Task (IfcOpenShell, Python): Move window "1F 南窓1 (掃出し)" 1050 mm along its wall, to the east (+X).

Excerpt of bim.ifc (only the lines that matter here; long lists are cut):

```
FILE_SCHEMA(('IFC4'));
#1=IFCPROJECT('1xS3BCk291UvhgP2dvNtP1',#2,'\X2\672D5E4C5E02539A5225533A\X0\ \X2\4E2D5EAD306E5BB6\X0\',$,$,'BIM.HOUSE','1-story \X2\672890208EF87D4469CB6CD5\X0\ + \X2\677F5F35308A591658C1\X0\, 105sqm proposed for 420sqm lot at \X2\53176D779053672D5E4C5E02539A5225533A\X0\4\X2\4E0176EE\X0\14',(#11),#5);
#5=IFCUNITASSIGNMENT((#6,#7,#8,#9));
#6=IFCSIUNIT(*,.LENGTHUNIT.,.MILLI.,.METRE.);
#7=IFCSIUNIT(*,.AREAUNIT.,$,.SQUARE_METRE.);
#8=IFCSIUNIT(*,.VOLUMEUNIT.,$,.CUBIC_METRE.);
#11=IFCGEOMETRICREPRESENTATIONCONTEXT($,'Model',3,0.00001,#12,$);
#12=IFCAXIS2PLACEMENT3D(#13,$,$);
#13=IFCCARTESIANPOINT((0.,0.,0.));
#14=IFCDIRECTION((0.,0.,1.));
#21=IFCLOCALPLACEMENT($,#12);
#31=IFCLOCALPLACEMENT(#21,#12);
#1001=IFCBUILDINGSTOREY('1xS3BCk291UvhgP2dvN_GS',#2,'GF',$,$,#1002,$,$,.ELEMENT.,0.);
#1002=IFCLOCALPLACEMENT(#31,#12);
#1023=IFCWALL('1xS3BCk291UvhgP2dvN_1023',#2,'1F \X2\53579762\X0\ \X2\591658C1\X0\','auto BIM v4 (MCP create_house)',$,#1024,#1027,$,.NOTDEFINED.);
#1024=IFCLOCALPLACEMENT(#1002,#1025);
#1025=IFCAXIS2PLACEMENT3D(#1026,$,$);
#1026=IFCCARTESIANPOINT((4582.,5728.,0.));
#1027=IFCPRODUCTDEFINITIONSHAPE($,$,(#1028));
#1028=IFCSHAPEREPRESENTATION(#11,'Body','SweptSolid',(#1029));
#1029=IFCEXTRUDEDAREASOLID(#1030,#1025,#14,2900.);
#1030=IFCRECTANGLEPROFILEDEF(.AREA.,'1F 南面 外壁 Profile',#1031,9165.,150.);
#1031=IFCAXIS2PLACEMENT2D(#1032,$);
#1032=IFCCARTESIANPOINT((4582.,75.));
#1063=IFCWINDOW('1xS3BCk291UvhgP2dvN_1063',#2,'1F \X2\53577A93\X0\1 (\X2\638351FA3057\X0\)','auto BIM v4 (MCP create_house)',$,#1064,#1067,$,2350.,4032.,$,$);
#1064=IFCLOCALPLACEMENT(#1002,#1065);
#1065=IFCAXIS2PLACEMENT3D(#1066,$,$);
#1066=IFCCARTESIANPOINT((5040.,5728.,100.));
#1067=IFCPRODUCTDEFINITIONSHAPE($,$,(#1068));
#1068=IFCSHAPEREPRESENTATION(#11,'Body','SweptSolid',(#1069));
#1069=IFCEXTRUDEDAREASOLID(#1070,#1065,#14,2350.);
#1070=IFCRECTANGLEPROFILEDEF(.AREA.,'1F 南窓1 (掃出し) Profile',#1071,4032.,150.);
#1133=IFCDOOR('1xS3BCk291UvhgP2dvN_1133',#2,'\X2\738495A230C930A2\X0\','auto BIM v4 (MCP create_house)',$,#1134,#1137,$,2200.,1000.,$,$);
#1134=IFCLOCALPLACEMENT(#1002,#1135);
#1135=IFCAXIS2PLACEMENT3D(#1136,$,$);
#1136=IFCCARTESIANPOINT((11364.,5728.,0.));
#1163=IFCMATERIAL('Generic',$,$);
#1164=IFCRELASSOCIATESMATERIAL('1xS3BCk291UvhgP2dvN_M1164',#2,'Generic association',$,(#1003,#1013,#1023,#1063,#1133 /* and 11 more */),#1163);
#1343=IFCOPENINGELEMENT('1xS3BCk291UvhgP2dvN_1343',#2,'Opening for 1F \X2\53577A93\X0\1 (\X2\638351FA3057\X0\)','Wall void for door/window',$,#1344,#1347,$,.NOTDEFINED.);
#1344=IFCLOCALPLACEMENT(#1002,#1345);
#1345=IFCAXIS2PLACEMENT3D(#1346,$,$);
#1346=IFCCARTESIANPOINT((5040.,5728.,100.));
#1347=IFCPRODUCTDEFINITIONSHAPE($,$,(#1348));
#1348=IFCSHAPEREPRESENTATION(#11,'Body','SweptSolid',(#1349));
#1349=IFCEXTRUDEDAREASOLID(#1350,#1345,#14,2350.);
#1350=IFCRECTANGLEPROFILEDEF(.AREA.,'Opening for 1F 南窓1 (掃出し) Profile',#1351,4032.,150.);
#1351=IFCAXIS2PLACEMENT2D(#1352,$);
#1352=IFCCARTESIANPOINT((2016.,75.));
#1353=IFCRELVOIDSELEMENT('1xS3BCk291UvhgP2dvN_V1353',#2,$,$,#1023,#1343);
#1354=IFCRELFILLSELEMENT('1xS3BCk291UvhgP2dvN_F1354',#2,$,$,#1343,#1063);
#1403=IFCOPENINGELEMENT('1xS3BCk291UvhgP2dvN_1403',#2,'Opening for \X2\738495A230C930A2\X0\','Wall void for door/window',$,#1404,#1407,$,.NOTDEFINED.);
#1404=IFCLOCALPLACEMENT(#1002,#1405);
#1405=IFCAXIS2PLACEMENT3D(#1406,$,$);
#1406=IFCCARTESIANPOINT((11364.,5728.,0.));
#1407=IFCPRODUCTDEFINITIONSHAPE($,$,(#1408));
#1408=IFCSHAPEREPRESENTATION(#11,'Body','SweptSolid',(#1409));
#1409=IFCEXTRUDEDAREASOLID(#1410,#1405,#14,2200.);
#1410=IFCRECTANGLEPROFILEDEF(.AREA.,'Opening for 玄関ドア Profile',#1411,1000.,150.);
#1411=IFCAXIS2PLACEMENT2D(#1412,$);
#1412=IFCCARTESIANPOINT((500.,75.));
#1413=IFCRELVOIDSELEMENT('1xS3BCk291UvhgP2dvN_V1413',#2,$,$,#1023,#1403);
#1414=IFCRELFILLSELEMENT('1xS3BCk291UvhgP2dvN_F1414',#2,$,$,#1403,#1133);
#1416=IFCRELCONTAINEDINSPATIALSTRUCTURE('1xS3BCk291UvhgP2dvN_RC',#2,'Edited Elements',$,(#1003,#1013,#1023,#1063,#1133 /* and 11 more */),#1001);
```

```python
import ifcopenshell
import ifcopenshell.api.geometry
import ifcopenshell.util.placement
import ifcopenshell.util.unit

model = ifcopenshell.open("bim.ifc")
unit_scale = ifcopenshell.util.unit.calculate_unit_scale(model)

window = model.by_id(1063)
opening = window.FillsVoids[0].RelatingOpeningElement
wall = opening.VoidsElements[0].RelatingBuildingElement

wall_matrix = ifcopenshell.util.placement.get_local_placement(wall.ObjectPlacement)
shift = wall_matrix[:3, 0] * 1.05 / unit_scale
before = ifcopenshell.util.placement.get_local_placement(window.ObjectPlacement)[:3, 3].copy()

# The window is not placed relative to its opening, so move both.
for product in (opening, window):
    matrix = ifcopenshell.util.placement.get_local_placement(product.ObjectPlacement)
    matrix[:3, 3] += shift
    ifcopenshell.api.geometry.edit_object_placement(model, product=product, matrix=matrix, is_si=False)

after = ifcopenshell.util.placement.get_local_placement(window.ObjectPlacement)[:3, 3]
print("window moved by", (after - before).round(3) + 0.0)

model.write("bim_updated.ifc")
```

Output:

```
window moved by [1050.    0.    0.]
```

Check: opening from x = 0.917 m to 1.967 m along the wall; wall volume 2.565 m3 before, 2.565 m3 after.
